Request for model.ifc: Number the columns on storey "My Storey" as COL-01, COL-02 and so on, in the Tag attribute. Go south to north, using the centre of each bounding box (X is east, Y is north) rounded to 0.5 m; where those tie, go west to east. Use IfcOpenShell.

First a look at what the model holds.

```python
import ifcopenshell
import ifcopenshell.util.element
import ifcopenshell.util.placement

model = ifcopenshell.open("model.ifc")
print(model.schema)
storey = next(s for s in model.by_type("IfcBuildingStorey") if s.Name == "My Storey")
columns = [e for e in ifcopenshell.util.element.get_decomposition(storey) if e.is_a("IfcColumn")]
for e in sorted(columns, key=lambda e: e.id()):
    origin = ifcopenshell.util.placement.get_local_placement(e.ObjectPlacement)[:3, 3]
    print(e.id(), e.Tag, e.Name, origin.round(2) + 0.0, sep=" | ")
```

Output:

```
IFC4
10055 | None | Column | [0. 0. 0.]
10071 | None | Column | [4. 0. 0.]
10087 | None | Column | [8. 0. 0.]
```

```python
import ifcopenshell
import ifcopenshell.geom
import ifcopenshell.util.element
import ifcopenshell.util.shape

model = ifcopenshell.open("model.ifc")
settings = ifcopenshell.geom.settings()
settings.set("use-world-coords", True)


def centre(element):
    shape = ifcopenshell.geom.create_shape(settings, element)
    return ifcopenshell.util.shape.get_bbox_centroid(shape.geometry)


storey = next(s for s in model.by_type("IfcBuildingStorey") if s.Name == "My Storey")
columns = [e for e in ifcopenshell.util.element.get_decomposition(storey) if e.is_a("IfcColumn")]

# Insertion points can sit at a corner or the storey origin, so sort by the geometry (in metres).
centres = {e: centre(e) for e in columns}
columns.sort(key=lambda e: (round(centres[e][1] / 0.5), centres[e][0]))

for i, e in enumerate(columns, start=1):
    number = f"COL-{i:02d}"
    e.Tag = number
    print(e.id(), number)

model.write("model_rev.ifc")
```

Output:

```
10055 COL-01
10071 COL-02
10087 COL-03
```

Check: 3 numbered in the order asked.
